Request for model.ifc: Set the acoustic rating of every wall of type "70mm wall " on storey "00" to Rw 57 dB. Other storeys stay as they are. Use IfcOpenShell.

First a look at what the model holds.

```python
import ifcopenshell
import ifcopenshell.util.element

model = ifcopenshell.open("model.ifc")
print(model.schema)
storey = next(s for s in model.by_type("IfcBuildingStorey") if s.Name == "00")
walls = [e for e in ifcopenshell.util.element.get_decomposition(storey) if e.is_a("IfcWall")]
seen = {}
for e in walls:
    element_type = ifcopenshell.util.element.get_type(e)
    key = (element_type.Name if element_type != e and element_type else None, ifcopenshell.util.element.get_pset(e, "Pset_WallCommon", "AcousticRating"))
    seen[key] = seen.get(key, 0) + 1
for (name, value), count in sorted(seen.items(), key=str):
    print(count, "x", name, "|", value)
```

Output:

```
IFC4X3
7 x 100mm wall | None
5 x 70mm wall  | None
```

```python
import ifcopenshell
import ifcopenshell.api.pset
import ifcopenshell.util.element

model = ifcopenshell.open("model.ifc")

storey = next(s for s in model.by_type("IfcBuildingStorey") if s.Name == "00")
walls = [e for e in ifcopenshell.util.element.get_decomposition(storey) if e.is_a("IfcWall")]

count = 0
for e in walls:
    element_type = ifcopenshell.util.element.get_type(e)
    if element_type in (None, e) or element_type.Name != "70mm wall ":
        continue
    # add_pset returns the element's existing set when there is one.
    pset = ifcopenshell.api.pset.add_pset(model, product=e, name="Pset_WallCommon")
    ifcopenshell.api.pset.edit_pset(model, pset=pset, properties={"AcousticRating": "Rw 57 dB"})
    count += 1

print(count, "walls updated")

model.write("model_rev.ifc")
```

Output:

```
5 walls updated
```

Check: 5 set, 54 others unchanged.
